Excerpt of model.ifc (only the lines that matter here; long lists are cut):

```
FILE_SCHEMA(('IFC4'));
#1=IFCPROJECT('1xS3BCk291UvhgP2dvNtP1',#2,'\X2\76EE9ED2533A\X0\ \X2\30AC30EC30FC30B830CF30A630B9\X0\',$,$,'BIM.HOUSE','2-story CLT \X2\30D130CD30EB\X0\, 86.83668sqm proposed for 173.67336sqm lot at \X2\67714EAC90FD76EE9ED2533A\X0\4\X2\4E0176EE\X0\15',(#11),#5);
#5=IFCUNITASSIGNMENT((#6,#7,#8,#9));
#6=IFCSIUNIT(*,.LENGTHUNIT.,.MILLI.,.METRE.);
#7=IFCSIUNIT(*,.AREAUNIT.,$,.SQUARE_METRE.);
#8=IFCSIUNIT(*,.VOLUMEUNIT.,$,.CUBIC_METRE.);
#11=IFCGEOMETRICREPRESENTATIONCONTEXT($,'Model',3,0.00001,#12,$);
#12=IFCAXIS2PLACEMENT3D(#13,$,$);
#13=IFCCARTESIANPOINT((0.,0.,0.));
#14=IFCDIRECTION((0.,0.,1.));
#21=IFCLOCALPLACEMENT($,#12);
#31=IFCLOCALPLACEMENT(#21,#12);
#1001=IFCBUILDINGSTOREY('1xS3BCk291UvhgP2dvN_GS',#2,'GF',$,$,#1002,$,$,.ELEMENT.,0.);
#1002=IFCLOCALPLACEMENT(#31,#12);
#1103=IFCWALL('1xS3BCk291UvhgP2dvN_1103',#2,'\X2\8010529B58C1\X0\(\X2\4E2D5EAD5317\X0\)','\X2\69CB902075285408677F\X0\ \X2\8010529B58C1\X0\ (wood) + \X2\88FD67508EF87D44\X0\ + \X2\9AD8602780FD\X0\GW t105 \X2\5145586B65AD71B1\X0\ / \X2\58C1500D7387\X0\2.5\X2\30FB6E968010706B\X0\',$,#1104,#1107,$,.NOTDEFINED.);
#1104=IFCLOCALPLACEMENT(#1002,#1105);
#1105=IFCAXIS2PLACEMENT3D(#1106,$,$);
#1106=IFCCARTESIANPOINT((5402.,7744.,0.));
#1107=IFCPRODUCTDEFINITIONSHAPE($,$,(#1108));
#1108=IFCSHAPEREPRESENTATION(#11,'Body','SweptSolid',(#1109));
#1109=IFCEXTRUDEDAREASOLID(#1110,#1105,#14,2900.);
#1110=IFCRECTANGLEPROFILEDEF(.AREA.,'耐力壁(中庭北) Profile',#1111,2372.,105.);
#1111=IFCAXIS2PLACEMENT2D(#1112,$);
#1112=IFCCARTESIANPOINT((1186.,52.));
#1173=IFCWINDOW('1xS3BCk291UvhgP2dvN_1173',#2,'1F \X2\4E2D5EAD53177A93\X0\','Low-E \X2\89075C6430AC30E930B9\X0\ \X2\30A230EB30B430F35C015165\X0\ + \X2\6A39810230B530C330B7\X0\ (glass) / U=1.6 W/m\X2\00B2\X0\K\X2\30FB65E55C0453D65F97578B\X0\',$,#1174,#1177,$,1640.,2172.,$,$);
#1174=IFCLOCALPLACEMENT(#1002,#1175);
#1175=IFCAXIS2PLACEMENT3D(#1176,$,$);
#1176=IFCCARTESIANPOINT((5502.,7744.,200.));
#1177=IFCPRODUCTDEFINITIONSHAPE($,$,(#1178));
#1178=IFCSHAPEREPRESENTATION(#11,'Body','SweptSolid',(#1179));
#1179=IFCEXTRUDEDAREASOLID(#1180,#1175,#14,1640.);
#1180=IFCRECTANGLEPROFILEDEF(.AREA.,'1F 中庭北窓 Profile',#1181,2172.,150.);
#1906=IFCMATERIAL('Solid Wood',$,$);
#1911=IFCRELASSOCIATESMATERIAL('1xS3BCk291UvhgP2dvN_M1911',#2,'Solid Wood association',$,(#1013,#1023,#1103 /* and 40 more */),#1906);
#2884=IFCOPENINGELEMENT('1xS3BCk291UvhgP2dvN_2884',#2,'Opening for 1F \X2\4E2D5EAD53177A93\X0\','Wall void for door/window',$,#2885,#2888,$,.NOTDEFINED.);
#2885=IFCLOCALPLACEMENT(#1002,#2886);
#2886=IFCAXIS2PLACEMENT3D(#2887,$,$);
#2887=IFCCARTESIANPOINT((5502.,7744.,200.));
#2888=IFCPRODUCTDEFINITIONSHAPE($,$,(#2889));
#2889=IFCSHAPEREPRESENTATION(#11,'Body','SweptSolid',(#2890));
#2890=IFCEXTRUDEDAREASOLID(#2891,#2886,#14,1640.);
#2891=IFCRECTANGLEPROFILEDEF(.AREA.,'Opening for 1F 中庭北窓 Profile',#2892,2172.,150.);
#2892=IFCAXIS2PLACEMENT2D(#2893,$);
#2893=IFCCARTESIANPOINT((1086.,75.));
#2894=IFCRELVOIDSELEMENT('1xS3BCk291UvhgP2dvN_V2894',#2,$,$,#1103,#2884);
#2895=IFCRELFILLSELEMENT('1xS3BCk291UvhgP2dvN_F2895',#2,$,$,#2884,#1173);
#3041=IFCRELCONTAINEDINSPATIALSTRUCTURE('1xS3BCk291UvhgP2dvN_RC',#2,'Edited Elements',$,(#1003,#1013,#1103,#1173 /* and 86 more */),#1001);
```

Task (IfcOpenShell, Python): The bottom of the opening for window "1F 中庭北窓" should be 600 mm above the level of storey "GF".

```python
import numpy as np
import ifcopenshell
import ifcopenshell.api.geometry
import ifcopenshell.geom
import ifcopenshell.util.element
import ifcopenshell.util.placement
import ifcopenshell.util.shape
import ifcopenshell.util.unit

model = ifcopenshell.open("model.ifc")
unit_scale = ifcopenshell.util.unit.calculate_unit_scale(model)

window = model.by_guid("1xS3BCk291UvhgP2dvN_1173")
opening = window.FillsVoids[0].RelatingOpeningElement
storey = ifcopenshell.util.element.get_container(window, ifc_class="IfcBuildingStorey")
level = ifcopenshell.util.placement.get_local_placement(storey.ObjectPlacement)[2, 3]

# The opening's origin need not be at the sill, so measure its lowest point.
shape = ifcopenshell.geom.create_shape(ifcopenshell.geom.settings(), opening)
bottom = ifcopenshell.util.shape.get_shape_bottom_elevation(shape, shape.geometry) / unit_scale
dz = level + 0.6 / unit_scale - bottom

shift = np.array([0.0, 0.0, dz])
# The window is not placed relative to its opening, so move both.
for product in (opening, window):
    matrix = ifcopenshell.util.placement.get_local_placement(product.ObjectPlacement)
    matrix[:3, 3] += shift
    ifcopenshell.api.geometry.edit_object_placement(model, product=product, matrix=matrix, is_si=False)

print(f"moved by {dz * unit_scale:+.3f} m")

model.write("model_updated.ifc")
```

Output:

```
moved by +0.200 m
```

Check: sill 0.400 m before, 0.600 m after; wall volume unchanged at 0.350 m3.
